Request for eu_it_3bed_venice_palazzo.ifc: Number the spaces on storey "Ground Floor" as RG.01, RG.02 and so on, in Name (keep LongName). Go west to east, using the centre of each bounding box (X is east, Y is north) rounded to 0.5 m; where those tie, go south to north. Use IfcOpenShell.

First a look at what the model holds.

```python
import ifcopenshell
import ifcopenshell.util.element
import ifcopenshell.util.placement

model = ifcopenshell.open("eu_it_3bed_venice_palazzo.ifc")
print(model.schema)
storey = next(s for s in model.by_type("IfcBuildingStorey") if s.Name == "Ground Floor")
spaces = [e for e in ifcopenshell.util.element.get_decomposition(storey) if e.is_a("IfcSpace")]
for e in sorted(spaces, key=lambda e: e.id()):
    origin = ifcopenshell.util.placement.get_local_placement(e.ObjectPlacement)[:3, 3]
    print(e.id(), e.Name, e.LongName, origin.round(2) + 0.0, sep=" | ")
```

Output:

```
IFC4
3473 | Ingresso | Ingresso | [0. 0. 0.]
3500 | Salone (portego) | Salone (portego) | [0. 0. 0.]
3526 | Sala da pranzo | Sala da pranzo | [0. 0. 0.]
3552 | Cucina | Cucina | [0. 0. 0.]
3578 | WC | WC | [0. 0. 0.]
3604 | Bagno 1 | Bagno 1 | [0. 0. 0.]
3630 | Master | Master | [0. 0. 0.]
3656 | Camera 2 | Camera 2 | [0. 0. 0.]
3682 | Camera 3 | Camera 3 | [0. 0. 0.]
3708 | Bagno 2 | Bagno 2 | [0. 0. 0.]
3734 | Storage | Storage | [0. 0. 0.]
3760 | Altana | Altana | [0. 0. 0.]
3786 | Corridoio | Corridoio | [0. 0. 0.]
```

```python
import ifcopenshell
import ifcopenshell.geom
import ifcopenshell.util.element
import ifcopenshell.util.shape

model = ifcopenshell.open("eu_it_3bed_venice_palazzo.ifc")
settings = ifcopenshell.geom.settings()
settings.set("use-world-coords", True)


def centre(element):
    shape = ifcopenshell.geom.create_shape(settings, element)
    return ifcopenshell.util.shape.get_bbox_centroid(shape.geometry)


storey = next(s for s in model.by_type("IfcBuildingStorey") if s.Name == "Ground Floor")
spaces = [e for e in ifcopenshell.util.element.get_decomposition(storey) if e.is_a("IfcSpace")]

# Insertion points can sit at a corner or the storey origin, so sort by the geometry (in metres).
centres = {e: centre(e) for e in spaces}
spaces.sort(key=lambda e: (round(centres[e][0] / 0.5), centres[e][1]))

for i, e in enumerate(spaces, start=1):
    number = f"RG.{i:02d}"
    e.Name = number
    print(e.id(), number)

model.write("eu_it_3bed_venice_palazzo_edited.ifc")
```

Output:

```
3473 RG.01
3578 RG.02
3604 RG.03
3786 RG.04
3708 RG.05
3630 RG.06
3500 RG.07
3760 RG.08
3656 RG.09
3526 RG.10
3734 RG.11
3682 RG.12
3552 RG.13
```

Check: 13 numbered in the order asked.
